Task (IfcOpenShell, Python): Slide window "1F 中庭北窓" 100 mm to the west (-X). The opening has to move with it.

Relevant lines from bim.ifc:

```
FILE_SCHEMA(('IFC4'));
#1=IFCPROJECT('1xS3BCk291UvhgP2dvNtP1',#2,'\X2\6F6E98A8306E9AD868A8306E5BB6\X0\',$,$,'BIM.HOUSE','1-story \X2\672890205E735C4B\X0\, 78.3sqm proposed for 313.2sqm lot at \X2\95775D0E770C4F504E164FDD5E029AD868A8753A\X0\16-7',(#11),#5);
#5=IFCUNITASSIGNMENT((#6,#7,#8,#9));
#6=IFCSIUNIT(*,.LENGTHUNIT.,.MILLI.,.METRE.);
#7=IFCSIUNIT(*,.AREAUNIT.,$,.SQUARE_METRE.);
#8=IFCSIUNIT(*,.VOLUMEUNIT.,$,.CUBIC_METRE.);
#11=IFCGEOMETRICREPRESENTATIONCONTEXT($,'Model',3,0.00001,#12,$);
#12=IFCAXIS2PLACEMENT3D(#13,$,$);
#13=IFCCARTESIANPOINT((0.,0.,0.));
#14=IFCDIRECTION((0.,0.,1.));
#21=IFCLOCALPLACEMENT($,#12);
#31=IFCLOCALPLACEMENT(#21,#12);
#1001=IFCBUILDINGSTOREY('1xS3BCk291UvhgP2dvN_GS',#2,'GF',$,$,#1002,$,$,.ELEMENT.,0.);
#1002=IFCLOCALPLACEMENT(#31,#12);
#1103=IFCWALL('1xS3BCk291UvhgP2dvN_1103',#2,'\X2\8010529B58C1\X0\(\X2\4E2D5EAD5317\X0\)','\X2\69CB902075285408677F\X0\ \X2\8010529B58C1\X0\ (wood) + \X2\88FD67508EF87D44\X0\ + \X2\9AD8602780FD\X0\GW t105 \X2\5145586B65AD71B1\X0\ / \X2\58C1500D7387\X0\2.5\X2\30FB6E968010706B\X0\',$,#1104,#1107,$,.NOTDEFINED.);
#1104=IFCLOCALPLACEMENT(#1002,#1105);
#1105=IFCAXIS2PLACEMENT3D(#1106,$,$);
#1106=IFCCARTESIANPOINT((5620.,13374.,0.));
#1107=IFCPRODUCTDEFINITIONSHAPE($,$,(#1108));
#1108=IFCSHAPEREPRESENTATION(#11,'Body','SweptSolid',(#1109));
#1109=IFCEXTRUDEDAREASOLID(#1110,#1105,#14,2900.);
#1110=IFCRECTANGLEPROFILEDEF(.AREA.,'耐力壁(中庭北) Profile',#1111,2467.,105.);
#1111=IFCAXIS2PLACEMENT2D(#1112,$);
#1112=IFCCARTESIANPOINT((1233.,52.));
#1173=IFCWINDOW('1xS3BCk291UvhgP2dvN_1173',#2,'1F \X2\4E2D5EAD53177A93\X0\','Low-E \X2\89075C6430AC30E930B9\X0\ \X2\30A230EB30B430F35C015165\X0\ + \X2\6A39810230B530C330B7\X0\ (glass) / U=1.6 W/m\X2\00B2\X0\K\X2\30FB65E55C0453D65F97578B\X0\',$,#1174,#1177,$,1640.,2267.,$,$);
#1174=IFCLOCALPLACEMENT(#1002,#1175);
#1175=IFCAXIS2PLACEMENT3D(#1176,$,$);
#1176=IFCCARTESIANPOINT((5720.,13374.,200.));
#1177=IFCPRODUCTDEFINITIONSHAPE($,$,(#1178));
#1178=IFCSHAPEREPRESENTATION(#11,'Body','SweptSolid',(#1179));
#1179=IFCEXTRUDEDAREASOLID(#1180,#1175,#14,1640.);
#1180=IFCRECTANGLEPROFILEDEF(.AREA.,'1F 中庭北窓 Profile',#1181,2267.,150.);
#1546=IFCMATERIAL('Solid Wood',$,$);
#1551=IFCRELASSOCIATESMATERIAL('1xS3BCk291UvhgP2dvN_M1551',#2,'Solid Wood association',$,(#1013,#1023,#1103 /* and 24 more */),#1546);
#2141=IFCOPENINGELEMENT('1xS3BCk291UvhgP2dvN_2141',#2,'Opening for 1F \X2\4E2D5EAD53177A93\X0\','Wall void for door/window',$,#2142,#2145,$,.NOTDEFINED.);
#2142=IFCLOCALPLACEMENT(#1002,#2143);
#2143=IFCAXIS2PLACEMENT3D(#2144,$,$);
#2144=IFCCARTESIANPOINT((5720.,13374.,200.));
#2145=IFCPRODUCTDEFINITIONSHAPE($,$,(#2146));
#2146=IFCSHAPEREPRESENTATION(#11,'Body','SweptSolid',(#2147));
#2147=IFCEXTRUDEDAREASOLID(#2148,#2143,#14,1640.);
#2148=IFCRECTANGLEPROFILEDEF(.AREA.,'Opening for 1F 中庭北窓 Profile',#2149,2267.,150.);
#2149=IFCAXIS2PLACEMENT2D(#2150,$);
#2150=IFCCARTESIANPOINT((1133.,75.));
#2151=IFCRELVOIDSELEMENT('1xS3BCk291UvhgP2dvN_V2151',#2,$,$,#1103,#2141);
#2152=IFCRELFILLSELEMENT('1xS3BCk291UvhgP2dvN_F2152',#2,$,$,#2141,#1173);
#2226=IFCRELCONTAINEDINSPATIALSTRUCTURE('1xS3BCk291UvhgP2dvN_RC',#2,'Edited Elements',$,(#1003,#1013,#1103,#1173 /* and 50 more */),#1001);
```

```python
import ifcopenshell
import ifcopenshell.api.geometry
import ifcopenshell.util.placement
import ifcopenshell.util.unit

model = ifcopenshell.open("bim.ifc")
unit_scale = ifcopenshell.util.unit.calculate_unit_scale(model)

window = model.by_guid("1xS3BCk291UvhgP2dvN_1173")
opening = window.FillsVoids[0].RelatingOpeningElement
wall = opening.VoidsElements[0].RelatingBuildingElement

wall_matrix = ifcopenshell.util.placement.get_local_placement(wall.ObjectPlacement)
shift = wall_matrix[:3, 0] * -0.1 / unit_scale
before = ifcopenshell.util.placement.get_local_placement(window.ObjectPlacement)[:3, 3].copy()

# The window is not placed relative to its opening, so move both.
for product in (opening, window):
    matrix = ifcopenshell.util.placement.get_local_placement(product.ObjectPlacement)
    matrix[:3, 3] += shift
    ifcopenshell.api.geometry.edit_object_placement(model, product=product, matrix=matrix, is_si=False)

after = ifcopenshell.util.placement.get_local_placement(window.ObjectPlacement)[:3, 3]
print("window moved by", (after - before).round(3) + 0.0)

model.write("bim_updated.ifc")
```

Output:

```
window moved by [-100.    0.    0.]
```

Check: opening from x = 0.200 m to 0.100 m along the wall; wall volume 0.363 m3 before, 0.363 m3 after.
